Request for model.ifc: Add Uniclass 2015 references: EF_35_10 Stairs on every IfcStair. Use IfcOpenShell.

First a look at what the model holds.

```python
import ifcopenshell

model = ifcopenshell.open("model.ifc")
print(model.schema)
print("classifications:", [c.Name for c in model.by_type("IfcClassification")])
for ifc_class in ("IfcDoor", "IfcRoof", "IfcStair", "IfcWall", "IfcWindow"):
    print(ifc_class, len(model.by_type(ifc_class)))
```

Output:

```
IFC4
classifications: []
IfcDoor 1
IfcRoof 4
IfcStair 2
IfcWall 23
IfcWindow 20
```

```python
import ifcopenshell
import ifcopenshell.api.classification

model = ifcopenshell.open("model.ifc")

system = ifcopenshell.api.classification.add_classification(model, classification="Uniclass 2015")

codes = {
    "IfcStair": ("EF_35_10", "Stairs"),
}
for ifc_class, (code, name) in codes.items():
    products = model.by_type(ifc_class)
    ifcopenshell.api.classification.add_reference(
        model, products=products, classification=system, identification=code, name=name
    )
    print(code, len(products))

model.write("model-out.ifc")
```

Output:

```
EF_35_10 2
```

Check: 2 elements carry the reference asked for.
